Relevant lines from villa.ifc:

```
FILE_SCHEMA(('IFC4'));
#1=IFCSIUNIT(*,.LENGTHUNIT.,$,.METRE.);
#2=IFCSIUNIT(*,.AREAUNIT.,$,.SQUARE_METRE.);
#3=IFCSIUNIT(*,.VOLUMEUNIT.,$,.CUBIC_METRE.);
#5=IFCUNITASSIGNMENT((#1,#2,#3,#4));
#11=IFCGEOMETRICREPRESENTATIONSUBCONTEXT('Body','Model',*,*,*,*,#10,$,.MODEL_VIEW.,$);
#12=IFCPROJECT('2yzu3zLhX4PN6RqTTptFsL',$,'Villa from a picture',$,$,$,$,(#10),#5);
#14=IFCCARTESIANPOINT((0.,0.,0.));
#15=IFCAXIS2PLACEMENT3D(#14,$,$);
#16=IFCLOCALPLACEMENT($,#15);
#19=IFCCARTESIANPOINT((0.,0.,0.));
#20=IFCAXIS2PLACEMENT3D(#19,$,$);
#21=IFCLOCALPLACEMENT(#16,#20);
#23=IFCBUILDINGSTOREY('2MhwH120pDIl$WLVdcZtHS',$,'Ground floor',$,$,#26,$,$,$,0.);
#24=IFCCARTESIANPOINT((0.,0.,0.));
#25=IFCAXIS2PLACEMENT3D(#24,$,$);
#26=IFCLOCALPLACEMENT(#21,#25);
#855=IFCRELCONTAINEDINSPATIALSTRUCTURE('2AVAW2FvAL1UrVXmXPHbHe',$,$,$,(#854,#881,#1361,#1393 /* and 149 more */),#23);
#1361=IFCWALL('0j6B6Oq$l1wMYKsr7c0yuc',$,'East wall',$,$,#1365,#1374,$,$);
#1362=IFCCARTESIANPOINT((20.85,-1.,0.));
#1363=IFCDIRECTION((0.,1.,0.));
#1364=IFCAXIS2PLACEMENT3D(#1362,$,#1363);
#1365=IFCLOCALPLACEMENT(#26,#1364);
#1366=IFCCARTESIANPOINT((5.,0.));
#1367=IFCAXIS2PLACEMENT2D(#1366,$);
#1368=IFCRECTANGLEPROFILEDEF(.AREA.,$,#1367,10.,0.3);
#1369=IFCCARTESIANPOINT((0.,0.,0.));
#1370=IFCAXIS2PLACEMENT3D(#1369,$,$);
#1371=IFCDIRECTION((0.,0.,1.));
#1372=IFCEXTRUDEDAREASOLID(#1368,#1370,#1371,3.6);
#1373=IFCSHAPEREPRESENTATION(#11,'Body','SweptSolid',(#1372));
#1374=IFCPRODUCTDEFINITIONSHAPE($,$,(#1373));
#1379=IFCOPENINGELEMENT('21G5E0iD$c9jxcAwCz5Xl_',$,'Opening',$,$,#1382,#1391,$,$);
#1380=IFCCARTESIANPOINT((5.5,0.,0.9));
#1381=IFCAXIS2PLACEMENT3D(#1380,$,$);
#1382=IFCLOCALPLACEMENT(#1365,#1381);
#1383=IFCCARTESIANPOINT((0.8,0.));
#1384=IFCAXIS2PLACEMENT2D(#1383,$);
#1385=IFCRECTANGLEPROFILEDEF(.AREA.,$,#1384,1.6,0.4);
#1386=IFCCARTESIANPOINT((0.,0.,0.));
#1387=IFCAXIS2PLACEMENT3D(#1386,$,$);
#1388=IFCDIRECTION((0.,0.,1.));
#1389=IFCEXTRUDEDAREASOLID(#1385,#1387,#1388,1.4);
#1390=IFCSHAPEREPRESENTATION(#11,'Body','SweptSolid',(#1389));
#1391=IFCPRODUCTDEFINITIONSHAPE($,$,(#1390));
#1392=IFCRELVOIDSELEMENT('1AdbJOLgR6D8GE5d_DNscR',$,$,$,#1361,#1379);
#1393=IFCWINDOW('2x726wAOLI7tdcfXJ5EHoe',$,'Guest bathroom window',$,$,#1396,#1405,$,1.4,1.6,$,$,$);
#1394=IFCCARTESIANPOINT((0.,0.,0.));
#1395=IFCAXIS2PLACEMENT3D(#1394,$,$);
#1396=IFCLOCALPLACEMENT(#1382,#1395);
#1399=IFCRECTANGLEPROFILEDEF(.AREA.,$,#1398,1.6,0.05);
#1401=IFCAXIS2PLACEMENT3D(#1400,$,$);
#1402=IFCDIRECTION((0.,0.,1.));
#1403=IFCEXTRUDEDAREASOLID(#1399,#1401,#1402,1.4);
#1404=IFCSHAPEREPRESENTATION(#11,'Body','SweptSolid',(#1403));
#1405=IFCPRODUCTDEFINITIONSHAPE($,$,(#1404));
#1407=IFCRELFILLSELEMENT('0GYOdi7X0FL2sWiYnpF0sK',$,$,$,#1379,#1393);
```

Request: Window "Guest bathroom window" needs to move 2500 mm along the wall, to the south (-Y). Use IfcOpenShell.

```python
import ifcopenshell
import ifcopenshell.api.geometry
import ifcopenshell.util.placement

model = ifcopenshell.open("villa.ifc")

window = model.by_guid("2x726wAOLI7tdcfXJ5EHoe")
opening = window.FillsVoids[0].RelatingOpeningElement
wall = opening.VoidsElements[0].RelatingBuildingElement

wall_matrix = ifcopenshell.util.placement.get_local_placement(wall.ObjectPlacement)
shift = wall_matrix[:3, 0] * -2.5
before = ifcopenshell.util.placement.get_local_placement(window.ObjectPlacement)[:3, 3].copy()

# The window is placed relative to its opening, so it follows when the opening moves.
matrix = ifcopenshell.util.placement.get_local_placement(opening.ObjectPlacement)
matrix[:3, 3] += shift
ifcopenshell.api.geometry.edit_object_placement(
    model, product=opening, matrix=matrix, is_si=False, should_transform_children=True
)

after = ifcopenshell.util.placement.get_local_placement(window.ObjectPlacement)[:3, 3]
print("window moved by", (after - before).round(3) + 0.0)

model.write("villa_v2.ifc")
```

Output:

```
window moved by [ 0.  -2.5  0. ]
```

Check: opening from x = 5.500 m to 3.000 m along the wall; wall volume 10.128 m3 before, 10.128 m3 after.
